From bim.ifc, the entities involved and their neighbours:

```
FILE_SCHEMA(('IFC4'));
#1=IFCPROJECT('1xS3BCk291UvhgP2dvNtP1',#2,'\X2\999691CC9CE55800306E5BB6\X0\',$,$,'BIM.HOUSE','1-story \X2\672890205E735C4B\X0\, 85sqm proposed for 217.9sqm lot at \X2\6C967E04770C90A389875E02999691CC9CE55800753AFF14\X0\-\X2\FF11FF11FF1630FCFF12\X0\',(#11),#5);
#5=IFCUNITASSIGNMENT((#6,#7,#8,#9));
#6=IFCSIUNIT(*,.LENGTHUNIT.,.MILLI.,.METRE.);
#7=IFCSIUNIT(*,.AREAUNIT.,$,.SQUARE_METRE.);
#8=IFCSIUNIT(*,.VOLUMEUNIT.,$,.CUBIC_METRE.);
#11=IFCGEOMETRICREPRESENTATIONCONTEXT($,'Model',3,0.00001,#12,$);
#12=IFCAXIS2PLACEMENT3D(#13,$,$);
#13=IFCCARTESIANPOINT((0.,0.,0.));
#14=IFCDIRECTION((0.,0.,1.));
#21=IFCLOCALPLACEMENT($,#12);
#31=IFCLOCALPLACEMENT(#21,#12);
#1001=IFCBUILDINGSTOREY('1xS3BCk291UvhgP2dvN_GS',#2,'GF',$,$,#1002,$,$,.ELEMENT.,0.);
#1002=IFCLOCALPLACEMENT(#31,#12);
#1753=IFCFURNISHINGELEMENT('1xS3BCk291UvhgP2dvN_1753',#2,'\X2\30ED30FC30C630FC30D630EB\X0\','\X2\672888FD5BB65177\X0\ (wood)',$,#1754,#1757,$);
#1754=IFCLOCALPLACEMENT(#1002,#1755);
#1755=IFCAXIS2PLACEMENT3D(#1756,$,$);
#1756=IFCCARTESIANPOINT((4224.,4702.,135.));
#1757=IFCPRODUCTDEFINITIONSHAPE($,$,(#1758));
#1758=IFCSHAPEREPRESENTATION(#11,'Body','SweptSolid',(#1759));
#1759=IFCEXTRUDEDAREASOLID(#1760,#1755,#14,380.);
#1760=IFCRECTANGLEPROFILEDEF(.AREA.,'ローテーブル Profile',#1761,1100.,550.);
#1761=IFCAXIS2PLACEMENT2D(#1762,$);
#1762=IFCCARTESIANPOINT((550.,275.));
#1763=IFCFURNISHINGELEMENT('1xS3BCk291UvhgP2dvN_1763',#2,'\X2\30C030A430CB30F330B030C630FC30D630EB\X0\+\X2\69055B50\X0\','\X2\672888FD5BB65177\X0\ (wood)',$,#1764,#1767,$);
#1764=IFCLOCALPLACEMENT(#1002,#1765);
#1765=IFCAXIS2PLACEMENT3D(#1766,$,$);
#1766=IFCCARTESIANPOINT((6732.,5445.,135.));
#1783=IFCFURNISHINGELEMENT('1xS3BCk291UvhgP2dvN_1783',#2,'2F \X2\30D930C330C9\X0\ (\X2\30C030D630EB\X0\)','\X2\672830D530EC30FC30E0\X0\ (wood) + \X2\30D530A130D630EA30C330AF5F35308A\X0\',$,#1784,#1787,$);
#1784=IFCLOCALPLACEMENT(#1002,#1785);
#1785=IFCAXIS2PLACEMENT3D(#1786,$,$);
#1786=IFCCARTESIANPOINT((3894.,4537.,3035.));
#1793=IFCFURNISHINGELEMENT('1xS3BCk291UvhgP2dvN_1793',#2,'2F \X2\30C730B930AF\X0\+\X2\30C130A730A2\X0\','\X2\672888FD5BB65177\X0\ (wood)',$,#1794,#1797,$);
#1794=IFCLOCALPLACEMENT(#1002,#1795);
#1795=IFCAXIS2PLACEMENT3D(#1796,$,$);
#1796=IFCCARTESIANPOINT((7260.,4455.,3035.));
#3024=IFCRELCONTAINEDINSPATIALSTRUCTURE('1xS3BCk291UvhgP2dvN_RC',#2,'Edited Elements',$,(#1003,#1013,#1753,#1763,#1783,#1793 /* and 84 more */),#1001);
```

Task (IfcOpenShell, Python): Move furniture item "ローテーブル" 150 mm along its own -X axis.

```python
import ifcopenshell
import ifcopenshell.api.geometry
import ifcopenshell.util.placement
import ifcopenshell.util.unit

model = ifcopenshell.open("bim.ifc")
unit_scale = ifcopenshell.util.unit.calculate_unit_scale(model)

item = model.by_id(1753)
matrix = ifcopenshell.util.placement.get_local_placement(item.ObjectPlacement)
matrix[:3, 3] -= matrix[:3, 0] * 0.15 / unit_scale
ifcopenshell.api.geometry.edit_object_placement(model, product=item, matrix=matrix, is_si=False)

print(ifcopenshell.util.placement.get_local_placement(item.ObjectPlacement).round(3) + 0.0)

model.write("bim_updated.ifc")
```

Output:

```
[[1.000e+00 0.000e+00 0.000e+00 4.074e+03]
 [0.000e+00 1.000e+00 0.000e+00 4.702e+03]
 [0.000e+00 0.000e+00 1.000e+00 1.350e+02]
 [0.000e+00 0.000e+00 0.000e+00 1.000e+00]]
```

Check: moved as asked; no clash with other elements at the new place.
